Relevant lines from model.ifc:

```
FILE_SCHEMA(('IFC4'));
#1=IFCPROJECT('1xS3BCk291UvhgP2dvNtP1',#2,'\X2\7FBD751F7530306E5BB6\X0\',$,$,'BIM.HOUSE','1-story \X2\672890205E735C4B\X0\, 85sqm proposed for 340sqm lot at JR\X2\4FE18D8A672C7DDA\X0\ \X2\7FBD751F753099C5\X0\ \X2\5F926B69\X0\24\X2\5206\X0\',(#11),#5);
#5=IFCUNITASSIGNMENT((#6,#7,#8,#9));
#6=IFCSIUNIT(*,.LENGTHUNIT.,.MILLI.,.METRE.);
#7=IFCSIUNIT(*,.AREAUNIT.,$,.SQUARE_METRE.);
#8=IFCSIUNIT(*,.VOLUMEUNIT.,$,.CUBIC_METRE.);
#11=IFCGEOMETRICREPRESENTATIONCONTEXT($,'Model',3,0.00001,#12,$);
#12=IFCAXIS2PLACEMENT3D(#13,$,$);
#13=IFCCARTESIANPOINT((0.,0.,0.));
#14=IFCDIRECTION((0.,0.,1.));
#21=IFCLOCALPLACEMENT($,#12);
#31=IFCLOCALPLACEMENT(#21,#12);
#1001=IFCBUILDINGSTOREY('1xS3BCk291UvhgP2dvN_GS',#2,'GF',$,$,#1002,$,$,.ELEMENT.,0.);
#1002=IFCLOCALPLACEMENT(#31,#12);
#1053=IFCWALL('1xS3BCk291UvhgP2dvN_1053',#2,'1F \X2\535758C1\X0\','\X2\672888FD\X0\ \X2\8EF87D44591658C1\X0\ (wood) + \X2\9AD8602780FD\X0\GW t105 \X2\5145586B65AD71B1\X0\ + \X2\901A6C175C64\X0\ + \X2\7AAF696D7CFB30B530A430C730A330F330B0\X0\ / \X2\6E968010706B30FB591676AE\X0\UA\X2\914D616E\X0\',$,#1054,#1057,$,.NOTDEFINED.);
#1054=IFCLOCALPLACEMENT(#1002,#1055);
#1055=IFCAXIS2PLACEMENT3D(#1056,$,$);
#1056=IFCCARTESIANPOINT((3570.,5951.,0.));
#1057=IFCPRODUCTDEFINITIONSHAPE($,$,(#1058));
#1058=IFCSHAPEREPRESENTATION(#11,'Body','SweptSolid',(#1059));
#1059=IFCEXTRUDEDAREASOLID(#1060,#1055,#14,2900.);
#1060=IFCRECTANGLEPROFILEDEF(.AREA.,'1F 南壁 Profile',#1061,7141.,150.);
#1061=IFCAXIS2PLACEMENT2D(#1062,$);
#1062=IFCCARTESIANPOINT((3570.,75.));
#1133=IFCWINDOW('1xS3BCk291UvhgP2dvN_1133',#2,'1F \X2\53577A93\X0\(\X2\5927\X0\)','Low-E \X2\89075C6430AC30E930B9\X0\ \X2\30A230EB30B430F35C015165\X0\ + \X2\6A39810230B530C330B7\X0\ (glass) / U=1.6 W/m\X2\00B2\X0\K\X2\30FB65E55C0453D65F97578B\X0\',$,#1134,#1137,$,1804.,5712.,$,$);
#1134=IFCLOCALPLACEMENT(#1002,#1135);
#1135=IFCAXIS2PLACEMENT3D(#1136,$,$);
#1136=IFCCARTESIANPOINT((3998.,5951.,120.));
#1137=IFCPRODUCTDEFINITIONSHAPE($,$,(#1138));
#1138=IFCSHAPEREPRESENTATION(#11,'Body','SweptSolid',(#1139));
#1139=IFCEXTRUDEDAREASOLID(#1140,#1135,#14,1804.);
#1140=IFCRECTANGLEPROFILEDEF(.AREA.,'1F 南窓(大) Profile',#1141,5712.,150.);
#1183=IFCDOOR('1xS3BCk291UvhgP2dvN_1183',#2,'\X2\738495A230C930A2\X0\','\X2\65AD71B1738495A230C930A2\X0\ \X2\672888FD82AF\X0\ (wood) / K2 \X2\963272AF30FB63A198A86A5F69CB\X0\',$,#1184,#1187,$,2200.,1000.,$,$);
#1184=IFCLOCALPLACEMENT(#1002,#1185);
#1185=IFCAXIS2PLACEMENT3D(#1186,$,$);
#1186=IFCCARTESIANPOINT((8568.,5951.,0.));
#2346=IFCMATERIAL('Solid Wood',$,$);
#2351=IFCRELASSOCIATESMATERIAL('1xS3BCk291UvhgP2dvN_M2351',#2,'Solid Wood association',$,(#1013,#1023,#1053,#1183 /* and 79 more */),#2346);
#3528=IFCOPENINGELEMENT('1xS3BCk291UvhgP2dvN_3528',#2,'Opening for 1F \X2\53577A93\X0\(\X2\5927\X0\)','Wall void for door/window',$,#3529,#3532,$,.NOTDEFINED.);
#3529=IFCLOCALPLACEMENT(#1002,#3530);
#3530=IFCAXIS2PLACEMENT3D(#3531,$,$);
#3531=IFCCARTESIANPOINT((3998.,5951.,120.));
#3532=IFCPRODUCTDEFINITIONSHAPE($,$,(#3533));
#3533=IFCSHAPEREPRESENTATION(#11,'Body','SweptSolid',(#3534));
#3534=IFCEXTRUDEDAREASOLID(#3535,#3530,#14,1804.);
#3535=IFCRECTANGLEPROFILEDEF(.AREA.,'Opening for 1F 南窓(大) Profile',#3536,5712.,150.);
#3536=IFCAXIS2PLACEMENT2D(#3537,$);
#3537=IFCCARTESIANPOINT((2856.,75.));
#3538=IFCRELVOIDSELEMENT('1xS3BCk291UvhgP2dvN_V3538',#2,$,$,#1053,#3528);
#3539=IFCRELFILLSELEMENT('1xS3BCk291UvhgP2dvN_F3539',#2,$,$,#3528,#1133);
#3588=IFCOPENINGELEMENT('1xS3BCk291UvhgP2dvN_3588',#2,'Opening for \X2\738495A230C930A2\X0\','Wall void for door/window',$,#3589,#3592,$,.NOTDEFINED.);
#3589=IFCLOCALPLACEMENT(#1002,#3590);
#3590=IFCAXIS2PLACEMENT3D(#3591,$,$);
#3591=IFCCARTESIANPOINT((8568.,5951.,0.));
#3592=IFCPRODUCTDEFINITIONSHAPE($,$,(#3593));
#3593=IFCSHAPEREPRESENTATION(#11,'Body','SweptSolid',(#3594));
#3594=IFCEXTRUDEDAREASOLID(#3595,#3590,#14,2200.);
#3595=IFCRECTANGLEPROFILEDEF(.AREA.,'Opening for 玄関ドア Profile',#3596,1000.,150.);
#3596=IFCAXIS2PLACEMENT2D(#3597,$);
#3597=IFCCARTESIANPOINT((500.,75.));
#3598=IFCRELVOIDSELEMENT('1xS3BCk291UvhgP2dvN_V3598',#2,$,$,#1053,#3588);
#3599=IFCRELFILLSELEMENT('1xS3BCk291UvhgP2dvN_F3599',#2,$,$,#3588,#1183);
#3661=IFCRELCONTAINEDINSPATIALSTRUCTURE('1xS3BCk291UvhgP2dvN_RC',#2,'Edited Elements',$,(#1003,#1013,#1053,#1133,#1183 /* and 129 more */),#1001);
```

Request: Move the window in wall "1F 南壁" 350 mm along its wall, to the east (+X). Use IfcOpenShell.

```python
import ifcopenshell
import ifcopenshell.api.geometry
import ifcopenshell.util.placement
import ifcopenshell.util.unit

model = ifcopenshell.open("model.ifc")
unit_scale = ifcopenshell.util.unit.calculate_unit_scale(model)

window = model.by_guid("1xS3BCk291UvhgP2dvN_1133")
opening = window.FillsVoids[0].RelatingOpeningElement
wall = opening.VoidsElements[0].RelatingBuildingElement

wall_matrix = ifcopenshell.util.placement.get_local_placement(wall.ObjectPlacement)
shift = wall_matrix[:3, 0] * 0.35 / unit_scale
before = ifcopenshell.util.placement.get_local_placement(window.ObjectPlacement)[:3, 3].copy()

# The window is not placed relative to its opening, so move both.
for product in (opening, window):
    matrix = ifcopenshell.util.placement.get_local_placement(product.ObjectPlacement)
    matrix[:3, 3] += shift
    ifcopenshell.api.geometry.edit_object_placement(model, product=product, matrix=matrix, is_si=False)

after = ifcopenshell.util.placement.get_local_placement(window.ObjectPlacement)[:3, 3]
print("window moved by", (after - before).round(3) + 0.0)

model.write("model_rev.ifc")
```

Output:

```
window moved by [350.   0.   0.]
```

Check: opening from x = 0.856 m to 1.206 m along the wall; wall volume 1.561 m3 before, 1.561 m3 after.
